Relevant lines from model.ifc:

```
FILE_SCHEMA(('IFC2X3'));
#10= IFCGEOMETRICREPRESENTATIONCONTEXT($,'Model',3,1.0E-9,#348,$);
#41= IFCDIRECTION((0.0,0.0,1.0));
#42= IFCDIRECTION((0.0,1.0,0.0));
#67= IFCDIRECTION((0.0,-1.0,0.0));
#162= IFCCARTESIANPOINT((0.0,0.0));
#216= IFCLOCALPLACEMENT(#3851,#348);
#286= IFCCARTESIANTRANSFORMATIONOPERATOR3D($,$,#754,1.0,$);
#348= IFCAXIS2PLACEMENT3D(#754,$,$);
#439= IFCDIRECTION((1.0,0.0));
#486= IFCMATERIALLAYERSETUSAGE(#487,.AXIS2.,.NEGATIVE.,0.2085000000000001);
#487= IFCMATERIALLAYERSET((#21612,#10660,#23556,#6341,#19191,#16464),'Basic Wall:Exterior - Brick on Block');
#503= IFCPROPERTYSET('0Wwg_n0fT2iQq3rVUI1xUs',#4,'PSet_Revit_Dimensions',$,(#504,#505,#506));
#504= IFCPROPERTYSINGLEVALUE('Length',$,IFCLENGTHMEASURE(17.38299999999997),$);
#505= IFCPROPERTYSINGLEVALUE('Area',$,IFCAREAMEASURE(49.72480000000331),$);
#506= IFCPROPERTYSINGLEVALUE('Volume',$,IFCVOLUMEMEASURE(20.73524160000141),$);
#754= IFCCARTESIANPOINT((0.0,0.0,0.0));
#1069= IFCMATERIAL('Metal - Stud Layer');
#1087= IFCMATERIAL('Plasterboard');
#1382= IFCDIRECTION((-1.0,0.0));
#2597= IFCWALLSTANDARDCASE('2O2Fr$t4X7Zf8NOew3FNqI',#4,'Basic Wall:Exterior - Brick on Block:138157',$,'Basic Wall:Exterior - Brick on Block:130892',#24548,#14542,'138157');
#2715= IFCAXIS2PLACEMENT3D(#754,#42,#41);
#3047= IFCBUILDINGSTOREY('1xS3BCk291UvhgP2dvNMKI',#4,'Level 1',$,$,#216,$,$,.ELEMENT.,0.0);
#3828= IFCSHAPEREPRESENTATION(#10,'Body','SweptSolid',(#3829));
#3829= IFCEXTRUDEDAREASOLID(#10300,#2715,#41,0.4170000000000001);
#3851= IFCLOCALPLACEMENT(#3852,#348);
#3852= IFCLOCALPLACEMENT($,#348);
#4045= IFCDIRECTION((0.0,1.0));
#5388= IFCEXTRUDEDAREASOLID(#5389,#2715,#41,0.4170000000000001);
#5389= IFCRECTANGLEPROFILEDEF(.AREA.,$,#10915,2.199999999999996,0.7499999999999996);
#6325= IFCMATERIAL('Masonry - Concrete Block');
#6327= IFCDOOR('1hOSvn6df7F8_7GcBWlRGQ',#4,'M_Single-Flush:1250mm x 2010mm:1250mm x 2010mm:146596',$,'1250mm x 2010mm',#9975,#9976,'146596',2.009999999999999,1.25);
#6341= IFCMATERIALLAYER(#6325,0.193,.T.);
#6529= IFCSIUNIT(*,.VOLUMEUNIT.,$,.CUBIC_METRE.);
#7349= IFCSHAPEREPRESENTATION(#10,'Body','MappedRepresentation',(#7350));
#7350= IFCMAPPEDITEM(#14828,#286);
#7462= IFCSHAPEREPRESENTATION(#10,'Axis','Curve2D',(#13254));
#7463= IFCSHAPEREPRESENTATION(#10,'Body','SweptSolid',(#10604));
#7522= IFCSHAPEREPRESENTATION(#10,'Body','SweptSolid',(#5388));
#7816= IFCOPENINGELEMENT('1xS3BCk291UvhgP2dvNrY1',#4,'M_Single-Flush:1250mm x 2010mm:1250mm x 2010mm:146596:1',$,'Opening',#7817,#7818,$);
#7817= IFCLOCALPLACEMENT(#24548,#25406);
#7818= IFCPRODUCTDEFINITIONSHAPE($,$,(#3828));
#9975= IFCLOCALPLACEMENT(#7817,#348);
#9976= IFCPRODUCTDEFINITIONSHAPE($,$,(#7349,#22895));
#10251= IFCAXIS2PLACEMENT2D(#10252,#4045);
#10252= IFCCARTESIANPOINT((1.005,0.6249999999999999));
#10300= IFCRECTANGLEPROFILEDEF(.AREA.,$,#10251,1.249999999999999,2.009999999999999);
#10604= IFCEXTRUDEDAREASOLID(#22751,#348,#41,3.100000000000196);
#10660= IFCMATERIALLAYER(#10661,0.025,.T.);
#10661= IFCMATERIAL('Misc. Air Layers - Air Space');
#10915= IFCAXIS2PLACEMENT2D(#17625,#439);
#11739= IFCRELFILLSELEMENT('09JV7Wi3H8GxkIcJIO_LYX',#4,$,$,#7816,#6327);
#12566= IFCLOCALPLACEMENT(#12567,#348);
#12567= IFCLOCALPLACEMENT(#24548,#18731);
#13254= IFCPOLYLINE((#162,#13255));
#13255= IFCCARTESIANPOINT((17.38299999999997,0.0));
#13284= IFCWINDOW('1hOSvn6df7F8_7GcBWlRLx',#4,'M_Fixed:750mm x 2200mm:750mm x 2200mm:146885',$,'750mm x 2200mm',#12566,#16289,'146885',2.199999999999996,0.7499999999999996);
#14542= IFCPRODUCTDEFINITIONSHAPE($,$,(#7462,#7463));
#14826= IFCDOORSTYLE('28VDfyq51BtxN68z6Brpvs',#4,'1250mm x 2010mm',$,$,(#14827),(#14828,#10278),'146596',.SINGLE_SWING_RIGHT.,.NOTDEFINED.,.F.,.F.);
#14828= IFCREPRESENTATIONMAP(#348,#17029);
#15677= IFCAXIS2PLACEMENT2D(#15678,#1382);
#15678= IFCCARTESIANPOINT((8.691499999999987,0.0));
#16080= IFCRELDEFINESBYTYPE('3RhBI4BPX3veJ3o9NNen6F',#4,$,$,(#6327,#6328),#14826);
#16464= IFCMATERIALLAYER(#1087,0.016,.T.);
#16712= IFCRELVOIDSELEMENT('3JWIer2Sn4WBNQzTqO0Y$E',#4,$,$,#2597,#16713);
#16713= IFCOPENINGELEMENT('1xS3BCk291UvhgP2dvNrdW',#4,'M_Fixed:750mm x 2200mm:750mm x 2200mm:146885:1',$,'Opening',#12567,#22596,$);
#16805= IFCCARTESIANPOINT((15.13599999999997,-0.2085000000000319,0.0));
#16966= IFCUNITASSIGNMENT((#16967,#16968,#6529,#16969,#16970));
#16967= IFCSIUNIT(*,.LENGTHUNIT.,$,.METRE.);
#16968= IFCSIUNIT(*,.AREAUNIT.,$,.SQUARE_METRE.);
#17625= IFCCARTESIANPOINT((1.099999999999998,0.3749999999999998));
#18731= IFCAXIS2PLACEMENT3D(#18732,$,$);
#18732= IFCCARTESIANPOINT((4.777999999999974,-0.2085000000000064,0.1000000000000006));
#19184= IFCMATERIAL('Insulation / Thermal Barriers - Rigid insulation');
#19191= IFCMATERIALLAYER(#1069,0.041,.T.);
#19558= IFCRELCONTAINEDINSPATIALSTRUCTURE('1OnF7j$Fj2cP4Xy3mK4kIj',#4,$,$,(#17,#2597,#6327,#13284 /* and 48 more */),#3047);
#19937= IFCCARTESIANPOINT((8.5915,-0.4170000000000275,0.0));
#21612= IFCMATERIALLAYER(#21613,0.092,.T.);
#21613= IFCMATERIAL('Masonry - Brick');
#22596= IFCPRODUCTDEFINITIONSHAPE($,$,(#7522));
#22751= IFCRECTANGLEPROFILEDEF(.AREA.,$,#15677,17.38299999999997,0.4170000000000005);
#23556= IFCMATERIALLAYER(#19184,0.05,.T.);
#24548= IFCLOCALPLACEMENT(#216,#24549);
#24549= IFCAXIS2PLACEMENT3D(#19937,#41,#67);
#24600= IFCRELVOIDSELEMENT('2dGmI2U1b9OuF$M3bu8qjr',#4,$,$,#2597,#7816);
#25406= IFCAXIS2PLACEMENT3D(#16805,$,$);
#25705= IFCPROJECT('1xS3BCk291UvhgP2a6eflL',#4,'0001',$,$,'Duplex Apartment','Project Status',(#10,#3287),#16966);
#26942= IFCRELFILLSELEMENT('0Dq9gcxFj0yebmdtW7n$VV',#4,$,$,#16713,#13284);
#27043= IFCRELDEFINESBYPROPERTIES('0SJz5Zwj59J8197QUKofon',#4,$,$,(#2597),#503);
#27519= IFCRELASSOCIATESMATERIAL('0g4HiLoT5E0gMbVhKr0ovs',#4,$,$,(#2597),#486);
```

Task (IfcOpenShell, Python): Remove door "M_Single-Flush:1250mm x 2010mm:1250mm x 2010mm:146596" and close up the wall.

```python
import ifcopenshell
import ifcopenshell.api.feature
import ifcopenshell.api.pset
import ifcopenshell.api.root
import ifcopenshell.geom
import ifcopenshell.util.element
import ifcopenshell.util.shape
import ifcopenshell.util.unit

model = ifcopenshell.open("model.ifc")
area_scale = ifcopenshell.util.unit.calculate_unit_scale(model, "AREAUNIT")
volume_scale = ifcopenshell.util.unit.calculate_unit_scale(model, "VOLUMEUNIT")
settings = ifcopenshell.geom.settings()


def volume(element):
    """Net volume in cubic metres, openings subtracted."""
    shape = ifcopenshell.geom.create_shape(settings, element)
    return ifcopenshell.util.shape.get_volume(shape.geometry)


door = model.by_id(6327)
opening = door.FillsVoids[0].RelatingOpeningElement
wall = opening.VoidsElements[0].RelatingBuildingElement
before = volume(wall)

ifcopenshell.api.root.remove_product(model, product=door)
ifcopenshell.api.feature.remove_feature(model, feature=opening)

after = volume(wall)
thickness = 0.417  # wall thickness in metres

# Update the wall's stored quantities.
pset = model.by_id(ifcopenshell.util.element.get_pset(wall, "PSet_Revit_Dimensions", should_inherit=False)["id"])
ifcopenshell.api.pset.edit_pset(model, pset=pset, properties={
    "Area": model.create_entity("IfcAreaMeasure", after / thickness / area_scale),
    "Volume": model.create_entity("IfcVolumeMeasure", after / volume_scale),
})

print(f"wall volume {before:.3f} -> {after:.3f} m3")

model.write("model_v2.ifc")
```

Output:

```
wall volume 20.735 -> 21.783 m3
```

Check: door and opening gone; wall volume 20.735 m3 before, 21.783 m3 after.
